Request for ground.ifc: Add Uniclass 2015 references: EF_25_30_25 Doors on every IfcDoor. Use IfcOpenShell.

First a look at what the model holds.

```python
import ifcopenshell

model = ifcopenshell.open("ground.ifc")
print(model.schema)
print("classifications:", [c.Name for c in model.by_type("IfcClassification")])
for ifc_class in ("IfcDoor", "IfcRoof", "IfcStair", "IfcWall", "IfcWindow"):
    print(ifc_class, len(model.by_type(ifc_class)))
```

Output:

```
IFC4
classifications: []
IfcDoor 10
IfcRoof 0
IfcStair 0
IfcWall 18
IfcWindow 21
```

```python
import ifcopenshell
import ifcopenshell.api.classification

model = ifcopenshell.open("ground.ifc")

system = ifcopenshell.api.classification.add_classification(model, classification="Uniclass 2015")

codes = {
    "IfcDoor": ("EF_25_30_25", "Doors"),
}
for ifc_class, (code, name) in codes.items():
    products = model.by_type(ifc_class)
    ifcopenshell.api.classification.add_reference(
        model, products=products, classification=system, identification=code, name=name
    )
    print(code, len(products))

model.write("ground_updated.ifc")
```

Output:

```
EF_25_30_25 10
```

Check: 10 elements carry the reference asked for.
